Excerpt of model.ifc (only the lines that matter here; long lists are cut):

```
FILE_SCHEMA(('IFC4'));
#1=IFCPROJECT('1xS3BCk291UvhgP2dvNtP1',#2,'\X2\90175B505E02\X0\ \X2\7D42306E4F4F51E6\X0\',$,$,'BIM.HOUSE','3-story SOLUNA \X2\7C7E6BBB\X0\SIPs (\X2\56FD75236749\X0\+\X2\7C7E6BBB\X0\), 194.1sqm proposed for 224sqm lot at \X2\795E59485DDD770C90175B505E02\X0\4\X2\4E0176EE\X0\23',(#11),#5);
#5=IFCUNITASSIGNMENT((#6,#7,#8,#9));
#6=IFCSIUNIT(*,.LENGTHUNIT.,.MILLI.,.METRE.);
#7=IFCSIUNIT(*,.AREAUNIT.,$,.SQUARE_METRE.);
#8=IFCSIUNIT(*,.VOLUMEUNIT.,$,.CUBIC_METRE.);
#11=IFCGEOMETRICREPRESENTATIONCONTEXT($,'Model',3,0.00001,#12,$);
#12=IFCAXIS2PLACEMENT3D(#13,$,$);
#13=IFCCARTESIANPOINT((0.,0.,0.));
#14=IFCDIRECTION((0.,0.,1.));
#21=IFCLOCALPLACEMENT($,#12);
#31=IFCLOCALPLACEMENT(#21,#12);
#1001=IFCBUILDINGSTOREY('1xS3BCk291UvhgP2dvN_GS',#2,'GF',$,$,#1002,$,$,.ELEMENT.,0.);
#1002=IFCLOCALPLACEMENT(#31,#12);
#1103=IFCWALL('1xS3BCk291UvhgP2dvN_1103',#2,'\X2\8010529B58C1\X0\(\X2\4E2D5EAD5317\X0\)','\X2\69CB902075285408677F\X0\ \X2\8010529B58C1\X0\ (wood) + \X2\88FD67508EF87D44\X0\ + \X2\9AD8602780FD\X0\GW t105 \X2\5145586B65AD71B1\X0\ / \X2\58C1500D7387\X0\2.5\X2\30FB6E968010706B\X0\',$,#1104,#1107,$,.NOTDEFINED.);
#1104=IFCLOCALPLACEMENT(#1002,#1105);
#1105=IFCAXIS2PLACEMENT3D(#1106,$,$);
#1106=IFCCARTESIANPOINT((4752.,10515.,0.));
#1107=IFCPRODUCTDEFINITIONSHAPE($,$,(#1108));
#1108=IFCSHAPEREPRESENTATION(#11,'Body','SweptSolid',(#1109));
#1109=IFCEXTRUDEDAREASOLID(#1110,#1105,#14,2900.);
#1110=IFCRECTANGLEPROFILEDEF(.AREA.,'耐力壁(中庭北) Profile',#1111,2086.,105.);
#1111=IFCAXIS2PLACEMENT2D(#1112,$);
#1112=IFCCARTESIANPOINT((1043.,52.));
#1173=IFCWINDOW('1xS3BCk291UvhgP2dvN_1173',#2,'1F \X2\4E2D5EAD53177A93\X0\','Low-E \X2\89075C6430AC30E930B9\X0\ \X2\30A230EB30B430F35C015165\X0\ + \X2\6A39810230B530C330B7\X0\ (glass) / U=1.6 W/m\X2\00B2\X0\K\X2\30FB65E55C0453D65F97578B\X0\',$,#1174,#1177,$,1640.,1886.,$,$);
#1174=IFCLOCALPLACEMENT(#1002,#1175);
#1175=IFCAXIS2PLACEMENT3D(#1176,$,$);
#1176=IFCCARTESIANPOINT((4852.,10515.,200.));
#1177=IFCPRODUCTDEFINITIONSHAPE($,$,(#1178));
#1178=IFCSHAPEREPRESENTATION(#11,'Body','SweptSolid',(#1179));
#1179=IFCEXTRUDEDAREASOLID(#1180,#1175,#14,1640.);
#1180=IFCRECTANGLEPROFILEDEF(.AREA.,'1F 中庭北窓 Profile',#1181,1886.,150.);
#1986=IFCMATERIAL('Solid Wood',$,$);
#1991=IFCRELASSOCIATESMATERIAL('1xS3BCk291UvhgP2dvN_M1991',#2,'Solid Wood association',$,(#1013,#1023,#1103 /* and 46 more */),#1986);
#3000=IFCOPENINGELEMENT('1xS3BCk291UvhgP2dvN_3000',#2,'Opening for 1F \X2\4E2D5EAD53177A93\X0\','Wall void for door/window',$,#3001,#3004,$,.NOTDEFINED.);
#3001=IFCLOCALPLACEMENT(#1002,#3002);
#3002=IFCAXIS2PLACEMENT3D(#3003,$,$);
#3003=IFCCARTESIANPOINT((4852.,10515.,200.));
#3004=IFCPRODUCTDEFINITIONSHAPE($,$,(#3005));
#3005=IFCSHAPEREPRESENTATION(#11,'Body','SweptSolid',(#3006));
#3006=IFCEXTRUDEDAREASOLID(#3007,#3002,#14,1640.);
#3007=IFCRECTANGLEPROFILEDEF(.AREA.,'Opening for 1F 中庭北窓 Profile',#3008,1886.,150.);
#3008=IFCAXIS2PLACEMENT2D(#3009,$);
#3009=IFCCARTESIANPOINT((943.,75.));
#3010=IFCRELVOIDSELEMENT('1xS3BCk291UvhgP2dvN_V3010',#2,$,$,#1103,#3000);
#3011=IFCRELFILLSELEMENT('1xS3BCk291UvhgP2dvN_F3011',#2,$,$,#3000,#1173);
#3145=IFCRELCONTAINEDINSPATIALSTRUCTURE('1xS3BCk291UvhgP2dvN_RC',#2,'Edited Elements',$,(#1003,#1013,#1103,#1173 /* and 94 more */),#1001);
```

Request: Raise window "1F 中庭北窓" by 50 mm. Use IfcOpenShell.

```python
import numpy as np
import ifcopenshell
import ifcopenshell.api.geometry
import ifcopenshell.util.placement
import ifcopenshell.util.unit

model = ifcopenshell.open("model.ifc")
unit_scale = ifcopenshell.util.unit.calculate_unit_scale(model)

window = model.by_guid("1xS3BCk291UvhgP2dvN_1173")
opening = window.FillsVoids[0].RelatingOpeningElement
dz = 0.05 / unit_scale

shift = np.array([0.0, 0.0, dz])
# The window is not placed relative to its opening, so move both.
for product in (opening, window):
    matrix = ifcopenshell.util.placement.get_local_placement(product.ObjectPlacement)
    matrix[:3, 3] += shift
    ifcopenshell.api.geometry.edit_object_placement(model, product=product, matrix=matrix, is_si=False)

print(f"moved by {dz * unit_scale:+.3f} m")

model.write("model_updated.ifc")
```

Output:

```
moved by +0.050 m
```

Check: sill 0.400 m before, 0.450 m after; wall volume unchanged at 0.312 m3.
